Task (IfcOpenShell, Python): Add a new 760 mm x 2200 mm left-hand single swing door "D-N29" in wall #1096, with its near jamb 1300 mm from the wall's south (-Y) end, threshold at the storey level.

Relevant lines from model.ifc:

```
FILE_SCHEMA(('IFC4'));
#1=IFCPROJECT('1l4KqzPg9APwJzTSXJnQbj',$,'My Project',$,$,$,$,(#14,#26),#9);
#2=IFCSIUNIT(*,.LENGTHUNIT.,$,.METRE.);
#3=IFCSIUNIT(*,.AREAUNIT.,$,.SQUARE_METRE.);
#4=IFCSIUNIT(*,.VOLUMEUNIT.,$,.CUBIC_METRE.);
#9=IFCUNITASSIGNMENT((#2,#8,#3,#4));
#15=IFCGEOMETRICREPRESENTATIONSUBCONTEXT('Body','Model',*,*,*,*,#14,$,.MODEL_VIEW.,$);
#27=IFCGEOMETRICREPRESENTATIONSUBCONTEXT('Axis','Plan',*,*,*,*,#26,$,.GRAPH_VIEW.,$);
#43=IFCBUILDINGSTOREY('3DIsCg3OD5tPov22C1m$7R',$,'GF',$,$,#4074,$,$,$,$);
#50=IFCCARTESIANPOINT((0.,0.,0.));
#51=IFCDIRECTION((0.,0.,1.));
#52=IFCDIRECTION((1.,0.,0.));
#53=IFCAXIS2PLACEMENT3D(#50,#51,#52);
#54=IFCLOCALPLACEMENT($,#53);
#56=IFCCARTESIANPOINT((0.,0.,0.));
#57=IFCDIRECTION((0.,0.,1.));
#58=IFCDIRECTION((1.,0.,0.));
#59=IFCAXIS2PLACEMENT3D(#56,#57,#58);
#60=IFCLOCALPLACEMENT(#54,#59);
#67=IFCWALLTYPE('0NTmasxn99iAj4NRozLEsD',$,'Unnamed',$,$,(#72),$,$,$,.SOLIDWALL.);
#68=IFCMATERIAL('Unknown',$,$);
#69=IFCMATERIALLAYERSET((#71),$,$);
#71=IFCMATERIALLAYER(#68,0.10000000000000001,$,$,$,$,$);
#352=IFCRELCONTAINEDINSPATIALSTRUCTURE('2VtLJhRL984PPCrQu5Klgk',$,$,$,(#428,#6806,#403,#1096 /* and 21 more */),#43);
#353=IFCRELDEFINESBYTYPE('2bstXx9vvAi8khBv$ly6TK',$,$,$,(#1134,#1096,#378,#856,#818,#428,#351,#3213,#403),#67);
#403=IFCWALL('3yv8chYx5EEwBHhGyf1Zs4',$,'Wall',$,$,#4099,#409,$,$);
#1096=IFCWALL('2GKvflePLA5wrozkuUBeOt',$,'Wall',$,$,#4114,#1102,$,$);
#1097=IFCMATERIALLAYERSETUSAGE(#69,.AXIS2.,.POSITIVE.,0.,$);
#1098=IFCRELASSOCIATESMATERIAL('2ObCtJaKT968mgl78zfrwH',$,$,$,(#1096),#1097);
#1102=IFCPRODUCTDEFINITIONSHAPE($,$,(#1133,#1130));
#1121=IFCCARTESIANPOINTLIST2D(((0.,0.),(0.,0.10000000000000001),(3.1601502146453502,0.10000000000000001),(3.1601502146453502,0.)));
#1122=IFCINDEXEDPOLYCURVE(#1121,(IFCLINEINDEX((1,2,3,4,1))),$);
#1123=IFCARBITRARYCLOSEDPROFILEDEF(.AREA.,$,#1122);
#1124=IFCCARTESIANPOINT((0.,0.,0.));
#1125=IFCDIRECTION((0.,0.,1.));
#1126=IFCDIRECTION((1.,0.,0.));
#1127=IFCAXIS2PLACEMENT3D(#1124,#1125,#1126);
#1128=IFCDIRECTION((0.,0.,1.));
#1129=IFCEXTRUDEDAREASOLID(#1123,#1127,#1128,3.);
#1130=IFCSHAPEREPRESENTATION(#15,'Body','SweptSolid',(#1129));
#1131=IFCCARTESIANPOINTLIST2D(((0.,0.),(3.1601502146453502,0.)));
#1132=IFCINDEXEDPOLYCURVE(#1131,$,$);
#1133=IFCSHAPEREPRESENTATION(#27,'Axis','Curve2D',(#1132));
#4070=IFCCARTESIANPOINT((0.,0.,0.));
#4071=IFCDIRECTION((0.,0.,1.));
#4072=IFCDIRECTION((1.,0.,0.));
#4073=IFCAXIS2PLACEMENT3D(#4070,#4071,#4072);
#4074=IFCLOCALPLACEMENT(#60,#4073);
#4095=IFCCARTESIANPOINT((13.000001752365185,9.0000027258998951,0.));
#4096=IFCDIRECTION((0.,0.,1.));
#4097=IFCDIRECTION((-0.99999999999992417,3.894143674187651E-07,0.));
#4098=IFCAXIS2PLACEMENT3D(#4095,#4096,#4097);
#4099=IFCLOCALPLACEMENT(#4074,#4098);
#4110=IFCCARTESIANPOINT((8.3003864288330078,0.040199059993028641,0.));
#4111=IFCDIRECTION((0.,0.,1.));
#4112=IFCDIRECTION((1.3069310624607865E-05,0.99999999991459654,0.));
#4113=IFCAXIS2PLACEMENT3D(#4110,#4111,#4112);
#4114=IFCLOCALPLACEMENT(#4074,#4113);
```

```python
import numpy as np
import ifcopenshell
import ifcopenshell.api.feature
import ifcopenshell.api.geometry
import ifcopenshell.api.root
import ifcopenshell.api.spatial
import ifcopenshell.geom
import ifcopenshell.util.element
import ifcopenshell.util.placement
import ifcopenshell.util.representation
import ifcopenshell.util.shape
import ifcopenshell.util.unit

model = ifcopenshell.open("model.ifc")
unit_scale = ifcopenshell.util.unit.calculate_unit_scale(model)
settings = ifcopenshell.geom.settings()


def volume(element):
    """Net volume in cubic metres, openings subtracted."""
    shape = ifcopenshell.geom.create_shape(settings, element)
    return ifcopenshell.util.shape.get_volume(shape.geometry)


wall = model.by_guid("2GKvflePLA5wrozkuUBeOt")
storey = ifcopenshell.util.element.get_container(wall, ifc_class="IfcBuildingStorey")
context = ifcopenshell.util.representation.get_context(model, "Model", "Body", "MODEL_VIEW")
before = volume(wall)

width, height, from_end, sill = 0.76, 2.2, 1.3, 0.0  # metres

# The wall runs along its own X axis, and the end named is its -X end.
wall_shape = ifcopenshell.geom.create_shape(settings, wall)
x, y, z = ifcopenshell.util.shape.get_vertices(wall_shape.geometry).T
start = x.min() + from_end
face, thickness = float(y.min()), float(y.max() - y.min())
wall_matrix = ifcopenshell.util.placement.get_local_placement(wall.ObjectPlacement)
level = ifcopenshell.util.placement.get_local_placement(storey.ObjectPlacement)[2, 3]


def in_wall(x, y):
    """Placement at x, y metres in the wall's axes, at sill height."""
    matrix = wall_matrix.copy()
    matrix[:, 3] = wall_matrix @ np.array([x / unit_scale, y / unit_scale, 0.0, 1.0])
    matrix[2, 3] = level + sill / unit_scale
    return matrix


# Opening: a box that overshoots both wall faces by 50 mm.
opening = ifcopenshell.api.root.create_entity(model, ifc_class="IfcOpeningElement", predefined_type="OPENING")
box = ifcopenshell.api.geometry.add_wall_representation(
    model, context=context, length=width, height=height, thickness=thickness + 0.1
)
ifcopenshell.api.geometry.assign_representation(model, product=opening, representation=box)
ifcopenshell.api.geometry.edit_object_placement(model, product=opening, matrix=in_wall(start, face - 0.05), is_si=False)
ifcopenshell.api.feature.add_feature(model, feature=opening, element=wall)

door = ifcopenshell.api.root.create_entity(model, ifc_class="IfcDoor", name="D-N29", predefined_type="DOOR")
door.OverallWidth, door.OverallHeight = width / unit_scale, height / unit_scale
door.OperationType = "SINGLE_SWING_LEFT"
body = ifcopenshell.api.geometry.add_door_representation(
    model,
    context=context,
    overall_width=door.OverallWidth,
    overall_height=door.OverallHeight,
    operation_type="SINGLE_SWING_LEFT",
    lining_properties={"LiningDepth": thickness / unit_scale, "ThresholdDepth": thickness / unit_scale},
)
ifcopenshell.api.geometry.assign_representation(model, product=door, representation=body)
ifcopenshell.api.spatial.assign_container(model, products=[door], relating_structure=storey)
ifcopenshell.api.feature.add_filling(model, opening=opening, element=door)

# The lining spans the wall, so the door starts at the wall face.
ifcopenshell.api.geometry.edit_object_placement(model, product=door, matrix=in_wall(start, face), is_si=False)

after = volume(wall)

print(f"wall volume {before:.3f} -> {after:.3f} m3")

model.write("model_rev.ifc")
```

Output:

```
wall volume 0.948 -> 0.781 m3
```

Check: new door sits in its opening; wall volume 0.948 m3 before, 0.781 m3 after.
